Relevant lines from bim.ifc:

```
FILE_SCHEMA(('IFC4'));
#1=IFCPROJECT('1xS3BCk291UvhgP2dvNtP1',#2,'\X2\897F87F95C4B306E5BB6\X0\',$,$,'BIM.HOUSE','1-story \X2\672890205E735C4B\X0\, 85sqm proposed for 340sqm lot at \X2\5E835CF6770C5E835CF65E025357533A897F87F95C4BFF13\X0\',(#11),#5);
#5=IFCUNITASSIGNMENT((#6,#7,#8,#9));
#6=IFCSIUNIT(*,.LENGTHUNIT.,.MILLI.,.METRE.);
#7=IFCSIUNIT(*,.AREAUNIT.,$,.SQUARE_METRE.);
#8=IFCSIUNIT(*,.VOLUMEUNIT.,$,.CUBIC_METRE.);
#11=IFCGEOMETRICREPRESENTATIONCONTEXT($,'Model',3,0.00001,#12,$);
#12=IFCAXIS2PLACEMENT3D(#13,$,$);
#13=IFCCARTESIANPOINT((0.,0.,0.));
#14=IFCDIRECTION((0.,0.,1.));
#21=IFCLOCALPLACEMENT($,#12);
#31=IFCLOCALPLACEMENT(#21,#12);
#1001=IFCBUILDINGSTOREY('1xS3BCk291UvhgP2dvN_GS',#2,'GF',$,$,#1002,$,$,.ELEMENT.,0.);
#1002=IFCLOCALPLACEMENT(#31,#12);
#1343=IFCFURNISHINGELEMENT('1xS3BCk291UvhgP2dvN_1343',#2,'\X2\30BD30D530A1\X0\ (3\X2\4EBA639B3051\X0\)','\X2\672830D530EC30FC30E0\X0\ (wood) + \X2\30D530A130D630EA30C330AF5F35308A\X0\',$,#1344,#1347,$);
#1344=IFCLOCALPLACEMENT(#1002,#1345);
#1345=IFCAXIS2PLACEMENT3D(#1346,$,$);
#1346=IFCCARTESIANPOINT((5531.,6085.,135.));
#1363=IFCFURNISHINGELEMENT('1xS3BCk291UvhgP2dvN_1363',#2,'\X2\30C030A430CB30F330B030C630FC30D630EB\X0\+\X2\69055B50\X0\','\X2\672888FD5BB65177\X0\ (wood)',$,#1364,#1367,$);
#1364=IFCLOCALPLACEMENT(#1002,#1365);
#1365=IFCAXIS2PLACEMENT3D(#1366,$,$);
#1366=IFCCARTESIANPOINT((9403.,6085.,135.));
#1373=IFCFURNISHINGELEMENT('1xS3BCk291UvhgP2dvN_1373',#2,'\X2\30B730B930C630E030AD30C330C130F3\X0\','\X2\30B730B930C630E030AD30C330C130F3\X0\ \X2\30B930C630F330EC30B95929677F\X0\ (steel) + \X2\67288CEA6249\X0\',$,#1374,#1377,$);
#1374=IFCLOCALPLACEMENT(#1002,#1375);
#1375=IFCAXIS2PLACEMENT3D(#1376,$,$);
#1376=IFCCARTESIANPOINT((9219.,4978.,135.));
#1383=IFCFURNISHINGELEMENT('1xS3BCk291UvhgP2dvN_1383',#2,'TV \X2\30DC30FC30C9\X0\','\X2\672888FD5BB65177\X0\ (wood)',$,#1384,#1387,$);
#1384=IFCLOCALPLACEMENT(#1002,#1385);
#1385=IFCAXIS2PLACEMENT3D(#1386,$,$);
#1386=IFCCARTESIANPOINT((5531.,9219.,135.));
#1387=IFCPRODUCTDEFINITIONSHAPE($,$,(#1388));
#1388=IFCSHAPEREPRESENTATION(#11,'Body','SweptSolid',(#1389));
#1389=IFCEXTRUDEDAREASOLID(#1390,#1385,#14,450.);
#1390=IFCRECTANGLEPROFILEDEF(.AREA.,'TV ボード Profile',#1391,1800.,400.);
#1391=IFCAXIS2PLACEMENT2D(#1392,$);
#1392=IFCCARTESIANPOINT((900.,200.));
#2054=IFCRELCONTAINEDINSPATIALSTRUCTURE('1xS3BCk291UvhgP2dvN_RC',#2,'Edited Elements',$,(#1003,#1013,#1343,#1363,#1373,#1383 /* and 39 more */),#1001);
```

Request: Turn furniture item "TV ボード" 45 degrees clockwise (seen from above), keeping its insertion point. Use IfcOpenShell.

```python
import ifcopenshell
import ifcopenshell.api.geometry
import ifcopenshell.util.placement

model = ifcopenshell.open("bim.ifc")

item = model.by_id(1383)
matrix = ifcopenshell.util.placement.get_local_placement(item.ObjectPlacement)
matrix = matrix @ ifcopenshell.util.placement.rotation(-45, "Z")
ifcopenshell.api.geometry.edit_object_placement(model, product=item, matrix=matrix, is_si=False)

print(ifcopenshell.util.placement.get_local_placement(item.ObjectPlacement).round(3) + 0.0)

model.write("bim_edited.ifc")
```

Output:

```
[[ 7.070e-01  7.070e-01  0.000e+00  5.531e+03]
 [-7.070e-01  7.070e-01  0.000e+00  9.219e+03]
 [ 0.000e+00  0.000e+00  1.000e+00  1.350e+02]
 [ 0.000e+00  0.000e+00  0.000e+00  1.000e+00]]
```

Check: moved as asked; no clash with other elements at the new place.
